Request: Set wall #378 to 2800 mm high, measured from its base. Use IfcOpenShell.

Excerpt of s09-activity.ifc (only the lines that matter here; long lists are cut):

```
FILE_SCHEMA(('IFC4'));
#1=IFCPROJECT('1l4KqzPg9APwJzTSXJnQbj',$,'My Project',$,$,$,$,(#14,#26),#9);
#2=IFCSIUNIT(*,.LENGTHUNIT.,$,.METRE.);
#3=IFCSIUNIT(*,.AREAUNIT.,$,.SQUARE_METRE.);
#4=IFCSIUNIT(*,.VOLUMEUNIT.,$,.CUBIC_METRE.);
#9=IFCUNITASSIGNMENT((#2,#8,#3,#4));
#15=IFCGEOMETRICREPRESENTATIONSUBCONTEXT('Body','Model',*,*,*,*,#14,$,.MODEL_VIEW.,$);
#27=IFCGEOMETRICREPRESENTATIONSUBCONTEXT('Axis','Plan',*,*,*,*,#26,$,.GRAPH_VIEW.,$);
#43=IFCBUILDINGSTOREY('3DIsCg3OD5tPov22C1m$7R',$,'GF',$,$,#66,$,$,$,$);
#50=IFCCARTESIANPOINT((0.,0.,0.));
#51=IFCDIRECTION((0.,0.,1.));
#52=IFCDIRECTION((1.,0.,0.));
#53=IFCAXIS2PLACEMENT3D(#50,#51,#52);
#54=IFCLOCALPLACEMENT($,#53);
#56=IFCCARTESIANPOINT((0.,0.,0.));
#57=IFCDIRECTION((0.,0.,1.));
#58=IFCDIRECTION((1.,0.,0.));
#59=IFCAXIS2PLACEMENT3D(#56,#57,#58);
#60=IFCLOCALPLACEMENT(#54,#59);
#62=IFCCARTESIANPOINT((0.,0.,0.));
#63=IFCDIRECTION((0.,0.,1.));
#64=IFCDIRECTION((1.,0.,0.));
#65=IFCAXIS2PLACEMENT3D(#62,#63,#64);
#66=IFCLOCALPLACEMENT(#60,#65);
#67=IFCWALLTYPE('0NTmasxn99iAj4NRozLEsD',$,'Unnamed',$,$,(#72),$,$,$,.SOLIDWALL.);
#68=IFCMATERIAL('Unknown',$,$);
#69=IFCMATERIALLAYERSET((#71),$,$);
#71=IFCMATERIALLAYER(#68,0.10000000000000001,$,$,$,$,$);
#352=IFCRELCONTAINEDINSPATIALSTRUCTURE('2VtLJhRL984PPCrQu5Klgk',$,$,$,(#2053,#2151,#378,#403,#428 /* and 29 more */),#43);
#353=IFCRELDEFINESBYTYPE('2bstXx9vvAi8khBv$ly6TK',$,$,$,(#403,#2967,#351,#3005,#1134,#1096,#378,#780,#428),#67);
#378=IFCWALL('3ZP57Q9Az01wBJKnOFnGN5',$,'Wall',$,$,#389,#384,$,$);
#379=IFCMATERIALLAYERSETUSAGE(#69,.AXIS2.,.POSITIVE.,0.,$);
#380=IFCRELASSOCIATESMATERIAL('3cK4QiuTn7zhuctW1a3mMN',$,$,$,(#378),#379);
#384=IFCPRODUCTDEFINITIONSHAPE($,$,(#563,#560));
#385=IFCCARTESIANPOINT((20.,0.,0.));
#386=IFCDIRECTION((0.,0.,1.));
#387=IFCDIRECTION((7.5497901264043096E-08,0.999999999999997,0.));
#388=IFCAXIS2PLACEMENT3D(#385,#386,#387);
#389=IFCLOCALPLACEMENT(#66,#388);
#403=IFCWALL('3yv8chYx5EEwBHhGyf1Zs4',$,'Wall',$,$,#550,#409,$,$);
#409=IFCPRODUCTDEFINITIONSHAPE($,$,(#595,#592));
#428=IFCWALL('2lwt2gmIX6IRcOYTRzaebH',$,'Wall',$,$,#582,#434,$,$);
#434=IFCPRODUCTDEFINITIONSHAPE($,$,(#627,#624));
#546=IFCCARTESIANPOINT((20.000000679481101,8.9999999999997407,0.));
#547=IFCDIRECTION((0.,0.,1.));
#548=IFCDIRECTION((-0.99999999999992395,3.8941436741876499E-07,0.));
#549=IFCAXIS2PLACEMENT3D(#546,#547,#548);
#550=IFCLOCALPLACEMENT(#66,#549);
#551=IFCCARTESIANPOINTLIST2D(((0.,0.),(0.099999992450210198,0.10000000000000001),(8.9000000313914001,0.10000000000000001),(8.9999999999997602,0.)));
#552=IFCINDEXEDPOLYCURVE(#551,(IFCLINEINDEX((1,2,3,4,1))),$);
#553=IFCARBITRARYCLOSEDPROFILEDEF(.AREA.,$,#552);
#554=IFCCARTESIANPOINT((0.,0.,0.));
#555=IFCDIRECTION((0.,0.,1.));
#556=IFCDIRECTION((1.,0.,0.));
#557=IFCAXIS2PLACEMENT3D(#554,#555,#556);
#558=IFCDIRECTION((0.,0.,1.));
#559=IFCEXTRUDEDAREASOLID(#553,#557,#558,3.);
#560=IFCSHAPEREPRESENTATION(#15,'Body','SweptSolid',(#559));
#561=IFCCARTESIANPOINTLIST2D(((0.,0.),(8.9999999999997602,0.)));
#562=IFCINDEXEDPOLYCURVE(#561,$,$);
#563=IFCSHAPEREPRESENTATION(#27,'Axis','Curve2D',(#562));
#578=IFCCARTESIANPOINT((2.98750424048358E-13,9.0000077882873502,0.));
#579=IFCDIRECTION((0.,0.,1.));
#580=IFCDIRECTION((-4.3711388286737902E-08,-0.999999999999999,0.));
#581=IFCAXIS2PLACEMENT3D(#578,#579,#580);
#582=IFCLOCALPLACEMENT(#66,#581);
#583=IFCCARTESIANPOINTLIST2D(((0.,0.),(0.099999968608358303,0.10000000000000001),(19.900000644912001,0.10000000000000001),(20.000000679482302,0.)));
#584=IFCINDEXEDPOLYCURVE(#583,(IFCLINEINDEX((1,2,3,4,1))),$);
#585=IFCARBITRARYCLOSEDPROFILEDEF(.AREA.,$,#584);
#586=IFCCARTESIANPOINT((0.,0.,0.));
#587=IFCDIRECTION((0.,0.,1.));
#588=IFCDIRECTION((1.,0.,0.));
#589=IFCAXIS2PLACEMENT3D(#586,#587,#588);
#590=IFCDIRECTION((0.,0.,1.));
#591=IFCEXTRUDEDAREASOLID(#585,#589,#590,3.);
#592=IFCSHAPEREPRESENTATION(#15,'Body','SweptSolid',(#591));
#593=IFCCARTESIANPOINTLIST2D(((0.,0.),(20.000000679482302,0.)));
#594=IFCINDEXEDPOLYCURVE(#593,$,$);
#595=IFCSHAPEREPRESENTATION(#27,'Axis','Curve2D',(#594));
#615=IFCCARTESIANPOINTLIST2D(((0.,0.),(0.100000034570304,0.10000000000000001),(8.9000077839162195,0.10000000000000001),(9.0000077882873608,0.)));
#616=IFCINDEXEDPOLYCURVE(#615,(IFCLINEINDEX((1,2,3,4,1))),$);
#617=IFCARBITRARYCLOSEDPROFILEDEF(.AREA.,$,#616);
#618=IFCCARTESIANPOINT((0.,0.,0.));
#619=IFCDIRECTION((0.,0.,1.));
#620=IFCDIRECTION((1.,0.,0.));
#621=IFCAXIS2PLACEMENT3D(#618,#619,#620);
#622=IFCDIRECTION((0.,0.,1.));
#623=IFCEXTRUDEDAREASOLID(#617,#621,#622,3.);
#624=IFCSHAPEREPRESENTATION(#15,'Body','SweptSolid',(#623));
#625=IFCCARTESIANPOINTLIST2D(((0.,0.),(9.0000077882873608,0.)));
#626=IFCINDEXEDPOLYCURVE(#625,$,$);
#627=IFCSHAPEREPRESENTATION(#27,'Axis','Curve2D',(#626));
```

```python
import ifcopenshell
import ifcopenshell.geom
import ifcopenshell.util.representation
import ifcopenshell.util.shape

model = ifcopenshell.open("s09-activity.ifc")
settings = ifcopenshell.geom.settings()


def volume(element):
    """Net volume in cubic metres, openings subtracted."""
    shape = ifcopenshell.geom.create_shape(settings, element)
    return ifcopenshell.util.shape.get_volume(shape.geometry)


wall = model.by_id(378)
before = volume(wall)

body = ifcopenshell.util.representation.get_representation(wall, "Model", "Body")
solid = body.Items[0]
old_height = solid.Depth
solid.Depth = 2.8
after = volume(wall)

print(f"height {old_height:g} -> {solid.Depth:g}, volume {before:.3f} -> {after:.3f} m3")

model.write("s09-activity_edited.ifc")
```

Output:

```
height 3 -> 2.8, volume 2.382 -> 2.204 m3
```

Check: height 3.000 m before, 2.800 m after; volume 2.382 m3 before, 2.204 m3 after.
